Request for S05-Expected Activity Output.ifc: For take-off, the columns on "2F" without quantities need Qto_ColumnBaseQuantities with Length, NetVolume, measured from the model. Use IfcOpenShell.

First a look at what the model holds.

```python
import ifcopenshell
import ifcopenshell.util.element
import ifcopenshell.util.unit

model = ifcopenshell.open("S05-Expected Activity Output.ifc")
print(model.schema)
for unit_type in ("LENGTHUNIT", "AREAUNIT", "VOLUMEUNIT"):
    print(unit_type, ifcopenshell.util.unit.calculate_unit_scale(model, unit_type))
storey = next(s for s in model.by_type("IfcBuildingStorey") if s.Name == "2F")
columns = [e for e in ifcopenshell.util.element.get_decomposition(storey) if e.is_a("IfcColumn")]
for e in sorted(columns, key=lambda e: e.id()):
    print(e.id(), e.is_a(), e.Name, list(ifcopenshell.util.element.get_psets(e, qtos_only=True)), sep=" | ")
```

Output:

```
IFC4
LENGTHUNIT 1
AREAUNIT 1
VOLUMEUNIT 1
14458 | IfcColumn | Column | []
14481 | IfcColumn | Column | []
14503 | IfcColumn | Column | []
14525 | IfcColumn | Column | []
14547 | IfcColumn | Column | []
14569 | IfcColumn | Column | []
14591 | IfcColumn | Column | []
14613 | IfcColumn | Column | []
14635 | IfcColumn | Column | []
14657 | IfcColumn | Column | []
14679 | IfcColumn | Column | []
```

```python
import ifcopenshell
import ifcopenshell.api.pset
import ifcopenshell.geom
import ifcopenshell.util.element
import ifcopenshell.util.shape
import ifcopenshell.util.unit

model = ifcopenshell.open("S05-Expected Activity Output.ifc")
unit_scale = ifcopenshell.util.unit.calculate_unit_scale(model)
volume_scale = ifcopenshell.util.unit.calculate_unit_scale(model, "VOLUMEUNIT")
settings = ifcopenshell.geom.settings()

storey = next(s for s in model.by_type("IfcBuildingStorey") if s.Name == "2F")
columns = [e for e in ifcopenshell.util.element.get_decomposition(storey) if e.is_a("IfcColumn")]

for e in sorted(columns, key=lambda e: e.id()):
    if ifcopenshell.util.element.get_psets(e, qtos_only=True, should_inherit=False):
        continue
    # Geometry comes back in metres, in the element's own axes.
    shape = ifcopenshell.geom.create_shape(settings, e)
    values = {
        "Length": ifcopenshell.util.shape.get_z(shape.geometry) / unit_scale,
        "NetVolume": ifcopenshell.util.shape.get_volume(shape.geometry) / volume_scale,
    }
    qto = ifcopenshell.api.pset.add_qto(model, product=e, name="Qto_ColumnBaseQuantities")
    ifcopenshell.api.pset.edit_qto(model, qto=qto, properties=values)
    print(e.id(), {k: round(v, 3) for k, v in values.items()})

model.write("S05-Expected Activity Output_v2.ifc")
```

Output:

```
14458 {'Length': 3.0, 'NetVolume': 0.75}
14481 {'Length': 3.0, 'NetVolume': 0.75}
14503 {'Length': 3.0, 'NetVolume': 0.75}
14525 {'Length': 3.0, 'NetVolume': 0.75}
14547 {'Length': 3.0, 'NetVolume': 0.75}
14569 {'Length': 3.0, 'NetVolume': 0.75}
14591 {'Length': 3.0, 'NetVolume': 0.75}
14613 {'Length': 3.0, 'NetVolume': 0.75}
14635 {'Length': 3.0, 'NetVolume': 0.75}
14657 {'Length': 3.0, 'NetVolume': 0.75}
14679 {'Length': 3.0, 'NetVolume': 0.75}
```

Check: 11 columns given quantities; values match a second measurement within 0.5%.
